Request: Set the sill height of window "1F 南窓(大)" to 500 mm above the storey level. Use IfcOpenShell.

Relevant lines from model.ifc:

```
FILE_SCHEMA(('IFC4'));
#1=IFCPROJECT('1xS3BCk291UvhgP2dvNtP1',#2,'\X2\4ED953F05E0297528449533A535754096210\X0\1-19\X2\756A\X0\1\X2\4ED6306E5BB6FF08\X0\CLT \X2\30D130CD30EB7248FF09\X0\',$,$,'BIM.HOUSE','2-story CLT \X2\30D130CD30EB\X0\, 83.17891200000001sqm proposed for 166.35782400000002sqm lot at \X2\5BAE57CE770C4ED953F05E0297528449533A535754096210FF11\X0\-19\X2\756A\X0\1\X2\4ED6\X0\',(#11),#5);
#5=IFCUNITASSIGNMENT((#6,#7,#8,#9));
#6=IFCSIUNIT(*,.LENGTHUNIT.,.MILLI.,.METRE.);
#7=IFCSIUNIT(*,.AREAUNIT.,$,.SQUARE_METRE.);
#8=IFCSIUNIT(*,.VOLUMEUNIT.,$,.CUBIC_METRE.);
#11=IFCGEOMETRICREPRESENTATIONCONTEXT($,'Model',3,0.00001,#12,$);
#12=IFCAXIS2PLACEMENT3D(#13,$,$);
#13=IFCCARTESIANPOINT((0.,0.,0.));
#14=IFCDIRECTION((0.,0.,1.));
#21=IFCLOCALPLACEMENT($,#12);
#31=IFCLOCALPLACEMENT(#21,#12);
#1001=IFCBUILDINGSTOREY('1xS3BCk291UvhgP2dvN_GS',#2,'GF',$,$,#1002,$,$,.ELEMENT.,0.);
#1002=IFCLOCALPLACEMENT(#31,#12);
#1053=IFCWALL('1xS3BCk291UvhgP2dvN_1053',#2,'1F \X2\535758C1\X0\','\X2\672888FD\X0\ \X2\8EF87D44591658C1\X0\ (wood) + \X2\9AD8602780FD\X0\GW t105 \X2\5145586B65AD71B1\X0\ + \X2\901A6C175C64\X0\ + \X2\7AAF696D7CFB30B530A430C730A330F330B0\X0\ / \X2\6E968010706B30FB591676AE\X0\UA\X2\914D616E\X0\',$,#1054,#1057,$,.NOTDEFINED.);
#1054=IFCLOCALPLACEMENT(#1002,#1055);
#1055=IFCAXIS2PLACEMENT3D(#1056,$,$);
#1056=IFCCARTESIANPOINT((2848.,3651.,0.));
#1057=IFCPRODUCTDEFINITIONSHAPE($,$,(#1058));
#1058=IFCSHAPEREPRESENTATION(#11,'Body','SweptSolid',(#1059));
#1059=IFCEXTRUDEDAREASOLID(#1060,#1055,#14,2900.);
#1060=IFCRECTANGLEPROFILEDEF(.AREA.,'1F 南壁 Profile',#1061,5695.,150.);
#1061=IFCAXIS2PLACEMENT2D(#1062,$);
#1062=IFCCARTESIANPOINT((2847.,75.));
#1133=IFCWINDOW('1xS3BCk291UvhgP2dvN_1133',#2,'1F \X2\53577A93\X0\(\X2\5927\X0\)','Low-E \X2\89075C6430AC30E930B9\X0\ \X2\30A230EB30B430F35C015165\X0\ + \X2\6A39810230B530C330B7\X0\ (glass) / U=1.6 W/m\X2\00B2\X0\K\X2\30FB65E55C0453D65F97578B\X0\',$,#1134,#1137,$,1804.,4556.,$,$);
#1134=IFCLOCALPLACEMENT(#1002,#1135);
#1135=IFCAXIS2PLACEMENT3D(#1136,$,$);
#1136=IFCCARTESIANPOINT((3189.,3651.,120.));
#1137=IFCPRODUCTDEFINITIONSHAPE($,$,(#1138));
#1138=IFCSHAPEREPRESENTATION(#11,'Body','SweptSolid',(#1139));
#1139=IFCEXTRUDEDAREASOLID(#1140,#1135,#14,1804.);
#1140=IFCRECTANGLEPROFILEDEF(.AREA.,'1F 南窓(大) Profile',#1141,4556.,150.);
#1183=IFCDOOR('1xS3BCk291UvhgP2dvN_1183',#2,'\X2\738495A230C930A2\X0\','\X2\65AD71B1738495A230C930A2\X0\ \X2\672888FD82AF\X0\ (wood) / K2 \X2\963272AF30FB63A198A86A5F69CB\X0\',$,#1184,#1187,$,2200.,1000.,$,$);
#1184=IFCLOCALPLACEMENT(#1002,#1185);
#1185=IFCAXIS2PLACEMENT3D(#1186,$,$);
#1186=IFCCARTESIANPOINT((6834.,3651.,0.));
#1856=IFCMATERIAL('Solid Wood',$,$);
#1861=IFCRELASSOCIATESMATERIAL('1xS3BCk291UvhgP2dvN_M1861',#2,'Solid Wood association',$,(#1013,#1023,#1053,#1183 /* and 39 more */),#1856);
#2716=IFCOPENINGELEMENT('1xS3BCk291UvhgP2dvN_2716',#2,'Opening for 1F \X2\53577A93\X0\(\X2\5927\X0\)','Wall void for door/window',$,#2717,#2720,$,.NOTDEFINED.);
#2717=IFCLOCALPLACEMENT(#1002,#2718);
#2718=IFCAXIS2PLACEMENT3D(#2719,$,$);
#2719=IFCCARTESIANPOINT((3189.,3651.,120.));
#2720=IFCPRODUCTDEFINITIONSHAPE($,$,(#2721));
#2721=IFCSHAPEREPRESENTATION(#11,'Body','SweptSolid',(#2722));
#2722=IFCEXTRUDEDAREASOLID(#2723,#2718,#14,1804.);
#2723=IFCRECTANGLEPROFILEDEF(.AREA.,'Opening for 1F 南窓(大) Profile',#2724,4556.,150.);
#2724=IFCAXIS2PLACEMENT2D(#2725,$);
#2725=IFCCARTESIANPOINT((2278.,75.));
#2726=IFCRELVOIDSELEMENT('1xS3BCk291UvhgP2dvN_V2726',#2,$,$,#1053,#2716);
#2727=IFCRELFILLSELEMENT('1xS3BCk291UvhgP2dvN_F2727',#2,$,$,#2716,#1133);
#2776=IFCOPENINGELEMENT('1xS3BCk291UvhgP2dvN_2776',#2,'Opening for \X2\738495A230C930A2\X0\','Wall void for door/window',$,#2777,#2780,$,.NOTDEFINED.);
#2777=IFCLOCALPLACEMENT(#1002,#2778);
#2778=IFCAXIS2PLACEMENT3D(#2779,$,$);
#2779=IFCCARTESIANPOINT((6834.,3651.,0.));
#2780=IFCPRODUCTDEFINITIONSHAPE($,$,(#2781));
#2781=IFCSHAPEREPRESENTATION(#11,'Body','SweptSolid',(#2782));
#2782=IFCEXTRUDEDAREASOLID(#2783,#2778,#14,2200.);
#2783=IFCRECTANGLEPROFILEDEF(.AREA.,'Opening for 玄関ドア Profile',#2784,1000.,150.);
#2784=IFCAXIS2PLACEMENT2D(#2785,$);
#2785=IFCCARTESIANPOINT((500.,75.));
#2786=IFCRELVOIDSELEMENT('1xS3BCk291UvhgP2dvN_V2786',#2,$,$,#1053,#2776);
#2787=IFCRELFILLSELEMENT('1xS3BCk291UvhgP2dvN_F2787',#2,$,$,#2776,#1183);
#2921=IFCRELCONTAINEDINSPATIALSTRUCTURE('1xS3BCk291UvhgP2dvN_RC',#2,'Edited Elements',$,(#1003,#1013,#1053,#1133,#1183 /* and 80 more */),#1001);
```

```python
import numpy as np
import ifcopenshell
import ifcopenshell.api.geometry
import ifcopenshell.geom
import ifcopenshell.util.element
import ifcopenshell.util.placement
import ifcopenshell.util.shape
import ifcopenshell.util.unit

model = ifcopenshell.open("model.ifc")
unit_scale = ifcopenshell.util.unit.calculate_unit_scale(model)

window = model.by_guid("1xS3BCk291UvhgP2dvN_1133")
opening = window.FillsVoids[0].RelatingOpeningElement
storey = ifcopenshell.util.element.get_container(window, ifc_class="IfcBuildingStorey")
level = ifcopenshell.util.placement.get_local_placement(storey.ObjectPlacement)[2, 3]

# The opening's origin need not be at the sill, so measure its lowest point.
shape = ifcopenshell.geom.create_shape(ifcopenshell.geom.settings(), opening)
bottom = ifcopenshell.util.shape.get_shape_bottom_elevation(shape, shape.geometry) / unit_scale
dz = level + 0.5 / unit_scale - bottom

shift = np.array([0.0, 0.0, dz])
# The window is not placed relative to its opening, so move both.
for product in (opening, window):
    matrix = ifcopenshell.util.placement.get_local_placement(product.ObjectPlacement)
    matrix[:3, 3] += shift
    ifcopenshell.api.geometry.edit_object_placement(model, product=product, matrix=matrix, is_si=False)

print(f"moved by {dz * unit_scale:+.3f} m")

model.write("model_v2.ifc")
```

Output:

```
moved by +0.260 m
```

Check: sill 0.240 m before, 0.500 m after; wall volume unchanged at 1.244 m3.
